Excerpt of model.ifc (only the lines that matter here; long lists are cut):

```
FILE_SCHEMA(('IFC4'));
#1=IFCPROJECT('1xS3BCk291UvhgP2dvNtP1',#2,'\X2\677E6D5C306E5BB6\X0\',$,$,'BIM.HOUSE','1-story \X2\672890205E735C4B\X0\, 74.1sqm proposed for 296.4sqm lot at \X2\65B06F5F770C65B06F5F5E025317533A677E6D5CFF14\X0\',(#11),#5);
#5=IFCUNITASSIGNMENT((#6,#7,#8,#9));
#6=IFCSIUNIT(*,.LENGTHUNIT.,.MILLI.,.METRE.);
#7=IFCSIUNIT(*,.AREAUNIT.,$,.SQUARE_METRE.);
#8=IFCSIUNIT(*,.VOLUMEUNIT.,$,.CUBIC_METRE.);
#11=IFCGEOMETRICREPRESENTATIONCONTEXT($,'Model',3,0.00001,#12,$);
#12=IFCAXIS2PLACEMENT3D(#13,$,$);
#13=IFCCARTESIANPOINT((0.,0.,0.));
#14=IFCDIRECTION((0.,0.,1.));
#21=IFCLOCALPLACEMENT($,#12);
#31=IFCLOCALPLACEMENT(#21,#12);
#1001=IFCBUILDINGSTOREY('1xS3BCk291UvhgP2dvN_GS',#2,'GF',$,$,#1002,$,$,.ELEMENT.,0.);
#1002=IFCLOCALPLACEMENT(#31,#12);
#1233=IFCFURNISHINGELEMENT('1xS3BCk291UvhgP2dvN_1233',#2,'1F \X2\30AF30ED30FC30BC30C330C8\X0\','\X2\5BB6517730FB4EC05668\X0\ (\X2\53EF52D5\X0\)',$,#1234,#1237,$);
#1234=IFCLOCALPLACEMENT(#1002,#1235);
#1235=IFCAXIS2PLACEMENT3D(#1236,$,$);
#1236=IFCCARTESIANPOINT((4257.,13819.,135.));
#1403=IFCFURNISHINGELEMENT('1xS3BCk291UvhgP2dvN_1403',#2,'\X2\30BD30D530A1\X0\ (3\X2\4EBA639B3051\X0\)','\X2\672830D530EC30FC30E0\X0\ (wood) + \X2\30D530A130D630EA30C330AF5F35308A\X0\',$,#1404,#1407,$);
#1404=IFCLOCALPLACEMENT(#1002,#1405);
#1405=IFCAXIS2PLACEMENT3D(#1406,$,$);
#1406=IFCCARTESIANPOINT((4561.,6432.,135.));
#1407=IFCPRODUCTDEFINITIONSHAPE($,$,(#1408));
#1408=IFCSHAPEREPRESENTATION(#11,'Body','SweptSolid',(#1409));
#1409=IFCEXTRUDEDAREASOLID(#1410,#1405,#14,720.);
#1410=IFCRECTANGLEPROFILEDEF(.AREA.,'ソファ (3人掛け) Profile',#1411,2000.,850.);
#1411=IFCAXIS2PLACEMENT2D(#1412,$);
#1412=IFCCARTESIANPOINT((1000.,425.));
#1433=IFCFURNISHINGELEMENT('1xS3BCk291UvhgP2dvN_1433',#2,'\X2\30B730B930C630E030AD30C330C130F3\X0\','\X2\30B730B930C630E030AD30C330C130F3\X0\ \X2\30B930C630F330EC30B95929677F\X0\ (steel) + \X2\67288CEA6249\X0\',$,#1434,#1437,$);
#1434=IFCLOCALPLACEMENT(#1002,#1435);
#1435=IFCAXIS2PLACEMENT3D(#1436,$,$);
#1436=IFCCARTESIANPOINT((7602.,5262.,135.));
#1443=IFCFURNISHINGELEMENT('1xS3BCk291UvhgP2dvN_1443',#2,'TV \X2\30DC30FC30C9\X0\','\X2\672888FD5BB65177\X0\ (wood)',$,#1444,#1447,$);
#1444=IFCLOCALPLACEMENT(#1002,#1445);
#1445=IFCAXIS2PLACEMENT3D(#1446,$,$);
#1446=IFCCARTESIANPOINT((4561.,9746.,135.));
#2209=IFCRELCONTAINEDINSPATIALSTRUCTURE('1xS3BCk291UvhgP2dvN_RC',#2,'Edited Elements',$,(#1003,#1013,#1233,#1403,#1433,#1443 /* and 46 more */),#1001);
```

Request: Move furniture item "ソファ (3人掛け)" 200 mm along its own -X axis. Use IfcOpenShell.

```python
import ifcopenshell
import ifcopenshell.api.geometry
import ifcopenshell.util.placement

model = ifcopenshell.open("model.ifc")

item = model.by_guid("1xS3BCk291UvhgP2dvN_1403")
matrix = ifcopenshell.util.placement.get_local_placement(item.ObjectPlacement)
matrix[:3, 3] -= matrix[:3, 0] * 200.0
ifcopenshell.api.geometry.edit_object_placement(model, product=item, matrix=matrix, is_si=False)

print(ifcopenshell.util.placement.get_local_placement(item.ObjectPlacement).round(3) + 0.0)

model.write("model_rev.ifc")
```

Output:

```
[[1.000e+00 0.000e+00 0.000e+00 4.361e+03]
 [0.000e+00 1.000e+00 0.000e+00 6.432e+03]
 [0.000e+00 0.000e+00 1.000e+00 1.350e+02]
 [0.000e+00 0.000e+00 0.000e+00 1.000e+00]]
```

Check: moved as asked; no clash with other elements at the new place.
